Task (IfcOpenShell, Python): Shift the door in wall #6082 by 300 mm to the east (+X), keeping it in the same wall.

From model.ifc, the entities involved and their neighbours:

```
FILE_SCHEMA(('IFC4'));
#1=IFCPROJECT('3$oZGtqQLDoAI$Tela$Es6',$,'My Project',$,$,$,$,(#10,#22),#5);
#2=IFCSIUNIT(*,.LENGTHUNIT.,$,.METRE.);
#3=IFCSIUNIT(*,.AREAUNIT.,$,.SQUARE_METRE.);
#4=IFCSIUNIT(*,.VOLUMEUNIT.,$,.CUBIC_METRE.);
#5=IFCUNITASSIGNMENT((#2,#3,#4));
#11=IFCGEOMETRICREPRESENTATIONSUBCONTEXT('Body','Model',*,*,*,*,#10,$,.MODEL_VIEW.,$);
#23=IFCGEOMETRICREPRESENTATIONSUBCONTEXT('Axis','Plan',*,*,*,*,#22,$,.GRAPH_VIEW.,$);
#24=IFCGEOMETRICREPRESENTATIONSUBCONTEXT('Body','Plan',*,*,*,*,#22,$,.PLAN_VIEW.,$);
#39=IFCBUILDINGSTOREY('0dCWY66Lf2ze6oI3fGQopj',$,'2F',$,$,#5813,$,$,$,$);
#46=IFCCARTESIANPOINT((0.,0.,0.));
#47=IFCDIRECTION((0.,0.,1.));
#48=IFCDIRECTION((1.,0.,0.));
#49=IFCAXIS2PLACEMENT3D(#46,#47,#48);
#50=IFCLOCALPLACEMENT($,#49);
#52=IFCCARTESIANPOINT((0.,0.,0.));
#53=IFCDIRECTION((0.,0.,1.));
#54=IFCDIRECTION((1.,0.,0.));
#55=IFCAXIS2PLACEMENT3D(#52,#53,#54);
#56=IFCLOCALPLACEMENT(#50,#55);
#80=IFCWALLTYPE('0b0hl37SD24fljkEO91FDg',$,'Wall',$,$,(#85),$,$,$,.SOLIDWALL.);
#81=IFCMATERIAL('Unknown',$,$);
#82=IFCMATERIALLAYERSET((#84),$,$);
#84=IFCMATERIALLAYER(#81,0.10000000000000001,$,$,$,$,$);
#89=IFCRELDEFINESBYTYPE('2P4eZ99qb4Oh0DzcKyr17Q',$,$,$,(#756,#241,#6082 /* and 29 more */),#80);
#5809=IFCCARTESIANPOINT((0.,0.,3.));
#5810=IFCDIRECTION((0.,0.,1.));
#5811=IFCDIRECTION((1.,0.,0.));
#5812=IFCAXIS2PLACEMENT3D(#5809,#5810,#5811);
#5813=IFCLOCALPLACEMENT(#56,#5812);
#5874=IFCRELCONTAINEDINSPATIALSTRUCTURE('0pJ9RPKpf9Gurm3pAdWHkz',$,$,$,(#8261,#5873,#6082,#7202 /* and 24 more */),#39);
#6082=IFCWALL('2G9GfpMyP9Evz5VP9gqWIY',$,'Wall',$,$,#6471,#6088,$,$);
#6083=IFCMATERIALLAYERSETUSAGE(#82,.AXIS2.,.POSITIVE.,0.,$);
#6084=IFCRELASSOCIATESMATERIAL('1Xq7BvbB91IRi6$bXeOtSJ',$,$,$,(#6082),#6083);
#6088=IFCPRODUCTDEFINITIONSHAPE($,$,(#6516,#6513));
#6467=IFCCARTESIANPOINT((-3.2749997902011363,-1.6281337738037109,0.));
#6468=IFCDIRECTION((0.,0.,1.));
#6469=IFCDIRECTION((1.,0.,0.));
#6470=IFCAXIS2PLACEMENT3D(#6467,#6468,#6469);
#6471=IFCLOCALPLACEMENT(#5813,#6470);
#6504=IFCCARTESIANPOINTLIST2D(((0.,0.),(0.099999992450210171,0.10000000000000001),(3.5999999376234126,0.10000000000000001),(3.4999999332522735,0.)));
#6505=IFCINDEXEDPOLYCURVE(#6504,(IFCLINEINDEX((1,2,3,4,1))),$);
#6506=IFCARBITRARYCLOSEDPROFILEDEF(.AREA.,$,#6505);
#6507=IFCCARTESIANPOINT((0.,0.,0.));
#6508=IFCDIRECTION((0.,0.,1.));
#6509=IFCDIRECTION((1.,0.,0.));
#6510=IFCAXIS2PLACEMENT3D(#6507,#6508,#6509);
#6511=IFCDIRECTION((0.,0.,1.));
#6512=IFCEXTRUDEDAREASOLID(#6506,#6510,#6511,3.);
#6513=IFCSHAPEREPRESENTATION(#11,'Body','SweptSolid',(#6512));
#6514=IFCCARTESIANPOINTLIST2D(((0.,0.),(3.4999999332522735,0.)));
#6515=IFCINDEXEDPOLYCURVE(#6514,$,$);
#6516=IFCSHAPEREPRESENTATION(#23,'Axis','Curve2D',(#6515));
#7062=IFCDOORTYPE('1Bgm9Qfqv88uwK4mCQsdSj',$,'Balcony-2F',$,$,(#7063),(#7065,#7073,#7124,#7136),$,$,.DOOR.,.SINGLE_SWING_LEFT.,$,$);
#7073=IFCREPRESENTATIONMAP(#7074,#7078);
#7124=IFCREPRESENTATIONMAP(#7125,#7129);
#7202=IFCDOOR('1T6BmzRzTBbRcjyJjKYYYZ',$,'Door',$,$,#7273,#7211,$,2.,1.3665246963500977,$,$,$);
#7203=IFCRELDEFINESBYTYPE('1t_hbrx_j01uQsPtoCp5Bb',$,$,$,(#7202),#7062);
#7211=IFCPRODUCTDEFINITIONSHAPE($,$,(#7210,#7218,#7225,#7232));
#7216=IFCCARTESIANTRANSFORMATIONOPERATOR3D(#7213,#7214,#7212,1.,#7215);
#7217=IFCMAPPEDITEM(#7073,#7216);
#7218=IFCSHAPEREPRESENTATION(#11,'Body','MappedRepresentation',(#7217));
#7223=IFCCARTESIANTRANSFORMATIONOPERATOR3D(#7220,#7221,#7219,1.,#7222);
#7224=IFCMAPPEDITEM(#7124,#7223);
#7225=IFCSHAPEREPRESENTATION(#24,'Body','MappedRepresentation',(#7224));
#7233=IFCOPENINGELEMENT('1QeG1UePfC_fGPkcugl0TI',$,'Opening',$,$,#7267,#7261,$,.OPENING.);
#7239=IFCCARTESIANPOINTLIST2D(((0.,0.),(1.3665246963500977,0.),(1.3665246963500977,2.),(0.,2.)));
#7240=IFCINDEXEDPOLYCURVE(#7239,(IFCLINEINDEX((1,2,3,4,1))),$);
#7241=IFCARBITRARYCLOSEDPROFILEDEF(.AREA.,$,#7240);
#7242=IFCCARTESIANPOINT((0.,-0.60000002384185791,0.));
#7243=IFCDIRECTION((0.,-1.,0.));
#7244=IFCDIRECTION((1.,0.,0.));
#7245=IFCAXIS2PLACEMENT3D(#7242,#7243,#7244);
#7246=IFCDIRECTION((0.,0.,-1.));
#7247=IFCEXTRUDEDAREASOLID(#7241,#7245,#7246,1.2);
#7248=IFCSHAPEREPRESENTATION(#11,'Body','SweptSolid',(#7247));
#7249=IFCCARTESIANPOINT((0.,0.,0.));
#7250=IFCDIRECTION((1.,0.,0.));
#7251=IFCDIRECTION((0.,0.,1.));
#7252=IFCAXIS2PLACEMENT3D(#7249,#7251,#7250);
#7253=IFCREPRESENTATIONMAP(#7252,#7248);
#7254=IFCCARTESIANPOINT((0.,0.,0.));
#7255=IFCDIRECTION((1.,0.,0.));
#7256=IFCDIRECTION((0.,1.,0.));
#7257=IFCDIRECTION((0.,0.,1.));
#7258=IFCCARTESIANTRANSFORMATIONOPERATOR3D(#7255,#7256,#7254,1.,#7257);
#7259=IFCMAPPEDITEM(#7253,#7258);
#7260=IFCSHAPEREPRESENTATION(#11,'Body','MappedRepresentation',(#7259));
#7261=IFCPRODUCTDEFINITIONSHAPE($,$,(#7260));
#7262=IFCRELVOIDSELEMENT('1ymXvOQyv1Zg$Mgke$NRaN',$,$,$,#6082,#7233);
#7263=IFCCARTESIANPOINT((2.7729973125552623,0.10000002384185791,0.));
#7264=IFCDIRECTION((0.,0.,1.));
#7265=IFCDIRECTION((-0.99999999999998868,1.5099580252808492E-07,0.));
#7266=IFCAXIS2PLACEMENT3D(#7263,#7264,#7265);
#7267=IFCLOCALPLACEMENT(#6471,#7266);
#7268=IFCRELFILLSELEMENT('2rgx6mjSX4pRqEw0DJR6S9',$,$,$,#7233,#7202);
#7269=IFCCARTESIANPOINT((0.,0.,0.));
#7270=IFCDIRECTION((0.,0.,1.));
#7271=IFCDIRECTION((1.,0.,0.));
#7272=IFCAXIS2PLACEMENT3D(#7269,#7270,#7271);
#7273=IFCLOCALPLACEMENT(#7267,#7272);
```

```python
import ifcopenshell
import ifcopenshell.api.geometry
import ifcopenshell.util.placement
import ifcopenshell.util.unit

model = ifcopenshell.open("model.ifc")
unit_scale = ifcopenshell.util.unit.calculate_unit_scale(model)

door = model.by_guid("1T6BmzRzTBbRcjyJjKYYYZ")
opening = door.FillsVoids[0].RelatingOpeningElement
wall = opening.VoidsElements[0].RelatingBuildingElement

wall_matrix = ifcopenshell.util.placement.get_local_placement(wall.ObjectPlacement)
shift = wall_matrix[:3, 0] * 0.3 / unit_scale
before = ifcopenshell.util.placement.get_local_placement(door.ObjectPlacement)[:3, 3].copy()

# The door is placed relative to its opening, so it follows when the opening moves.
matrix = ifcopenshell.util.placement.get_local_placement(opening.ObjectPlacement)
matrix[:3, 3] += shift
ifcopenshell.api.geometry.edit_object_placement(
    model, product=opening, matrix=matrix, is_si=False, should_transform_children=True
)

after = ifcopenshell.util.placement.get_local_placement(door.ObjectPlacement)[:3, 3]
print("door moved by", (after - before).round(3) + 0.0)

model.write("model_updated.ifc")
```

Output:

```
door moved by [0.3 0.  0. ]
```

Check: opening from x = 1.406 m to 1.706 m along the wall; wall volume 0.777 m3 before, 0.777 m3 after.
